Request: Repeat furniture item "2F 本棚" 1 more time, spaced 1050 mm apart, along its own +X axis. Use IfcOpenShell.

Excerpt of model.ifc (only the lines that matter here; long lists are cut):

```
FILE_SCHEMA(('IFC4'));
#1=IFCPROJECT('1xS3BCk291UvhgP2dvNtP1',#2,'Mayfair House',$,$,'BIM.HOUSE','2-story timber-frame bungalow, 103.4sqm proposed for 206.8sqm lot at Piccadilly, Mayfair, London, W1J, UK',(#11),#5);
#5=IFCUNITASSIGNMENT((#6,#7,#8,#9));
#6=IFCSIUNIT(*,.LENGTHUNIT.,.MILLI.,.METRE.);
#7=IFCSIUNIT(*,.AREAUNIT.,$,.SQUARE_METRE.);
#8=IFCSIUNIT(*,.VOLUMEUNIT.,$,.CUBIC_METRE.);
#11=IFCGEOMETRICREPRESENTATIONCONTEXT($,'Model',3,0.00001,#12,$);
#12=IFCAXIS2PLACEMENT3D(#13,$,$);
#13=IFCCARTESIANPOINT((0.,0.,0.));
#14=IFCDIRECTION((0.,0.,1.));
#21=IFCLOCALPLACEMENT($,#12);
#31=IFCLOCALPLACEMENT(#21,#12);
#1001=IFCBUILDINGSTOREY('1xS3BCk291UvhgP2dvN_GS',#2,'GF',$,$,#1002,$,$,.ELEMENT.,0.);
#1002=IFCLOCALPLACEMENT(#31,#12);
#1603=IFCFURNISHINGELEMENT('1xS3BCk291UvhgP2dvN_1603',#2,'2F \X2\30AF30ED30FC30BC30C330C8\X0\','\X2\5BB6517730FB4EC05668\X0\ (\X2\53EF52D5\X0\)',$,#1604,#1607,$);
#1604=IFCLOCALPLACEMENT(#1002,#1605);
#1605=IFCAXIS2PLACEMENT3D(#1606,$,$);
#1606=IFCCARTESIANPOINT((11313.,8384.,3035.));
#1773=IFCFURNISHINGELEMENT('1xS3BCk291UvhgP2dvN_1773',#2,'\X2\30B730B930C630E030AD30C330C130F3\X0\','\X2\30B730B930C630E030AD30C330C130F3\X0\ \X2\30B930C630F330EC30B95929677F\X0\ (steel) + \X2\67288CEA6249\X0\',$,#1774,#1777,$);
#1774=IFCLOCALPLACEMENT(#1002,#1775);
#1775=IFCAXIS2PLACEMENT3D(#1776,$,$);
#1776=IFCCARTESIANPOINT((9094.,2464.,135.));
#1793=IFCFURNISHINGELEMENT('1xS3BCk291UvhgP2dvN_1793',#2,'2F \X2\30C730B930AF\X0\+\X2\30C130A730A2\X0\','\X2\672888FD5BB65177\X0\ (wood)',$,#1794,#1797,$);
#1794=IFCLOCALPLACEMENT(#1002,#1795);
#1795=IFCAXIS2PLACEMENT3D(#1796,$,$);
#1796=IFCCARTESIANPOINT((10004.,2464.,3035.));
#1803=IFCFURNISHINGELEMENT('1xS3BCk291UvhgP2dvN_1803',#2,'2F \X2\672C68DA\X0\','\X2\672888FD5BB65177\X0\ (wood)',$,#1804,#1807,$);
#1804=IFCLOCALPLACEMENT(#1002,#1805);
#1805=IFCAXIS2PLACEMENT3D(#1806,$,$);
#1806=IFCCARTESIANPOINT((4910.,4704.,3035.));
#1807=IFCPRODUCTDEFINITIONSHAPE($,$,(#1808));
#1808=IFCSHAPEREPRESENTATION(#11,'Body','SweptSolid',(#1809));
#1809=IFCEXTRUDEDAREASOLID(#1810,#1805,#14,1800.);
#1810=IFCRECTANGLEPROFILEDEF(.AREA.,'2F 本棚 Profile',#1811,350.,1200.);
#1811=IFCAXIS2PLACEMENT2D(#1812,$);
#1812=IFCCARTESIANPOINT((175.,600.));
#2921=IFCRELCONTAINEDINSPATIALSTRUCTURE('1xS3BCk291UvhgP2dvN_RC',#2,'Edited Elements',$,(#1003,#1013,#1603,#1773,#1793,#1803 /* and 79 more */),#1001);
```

```python
import ifcopenshell
import ifcopenshell.api.geometry
import ifcopenshell.api.root
import ifcopenshell.util.element
import ifcopenshell.util.placement

model = ifcopenshell.open("model.ifc")


def reuse_history(source, copy):
    """copy_class also copies each property set's owner history, people and application; keep the originals."""
    for rel in copy.IsDefinedBy:
        if rel.is_a("IfcRelDefinesByProperties") and (history := rel.RelatingPropertyDefinition.OwnerHistory):
            rel.RelatingPropertyDefinition.OwnerHistory = source.OwnerHistory
            ifcopenshell.util.element.remove_deep2(model, history)


source = model.by_guid("1xS3BCk291UvhgP2dvN_1803")
base = ifcopenshell.util.placement.get_local_placement(source.ObjectPlacement)
step = base[:3, 0] * 1050.0

for i in range(1, 2):
    copy = ifcopenshell.api.root.copy_class(model, product=source)
    copy.Representation = ifcopenshell.util.element.copy_deep(
        model, source.Representation, exclude=["IfcGeometricRepresentationContext", "IfcRepresentationMap"]
    )
    reuse_history(source, copy)
    matrix = base.copy()
    matrix[:3, 3] += i * step
    print("added at", matrix[:3, 3].round(3) + 0.0)
    ifcopenshell.api.geometry.edit_object_placement(model, product=copy, matrix=matrix, is_si=False)

model.write("model-out.ifc")
```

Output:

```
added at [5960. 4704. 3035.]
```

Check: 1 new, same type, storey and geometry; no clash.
